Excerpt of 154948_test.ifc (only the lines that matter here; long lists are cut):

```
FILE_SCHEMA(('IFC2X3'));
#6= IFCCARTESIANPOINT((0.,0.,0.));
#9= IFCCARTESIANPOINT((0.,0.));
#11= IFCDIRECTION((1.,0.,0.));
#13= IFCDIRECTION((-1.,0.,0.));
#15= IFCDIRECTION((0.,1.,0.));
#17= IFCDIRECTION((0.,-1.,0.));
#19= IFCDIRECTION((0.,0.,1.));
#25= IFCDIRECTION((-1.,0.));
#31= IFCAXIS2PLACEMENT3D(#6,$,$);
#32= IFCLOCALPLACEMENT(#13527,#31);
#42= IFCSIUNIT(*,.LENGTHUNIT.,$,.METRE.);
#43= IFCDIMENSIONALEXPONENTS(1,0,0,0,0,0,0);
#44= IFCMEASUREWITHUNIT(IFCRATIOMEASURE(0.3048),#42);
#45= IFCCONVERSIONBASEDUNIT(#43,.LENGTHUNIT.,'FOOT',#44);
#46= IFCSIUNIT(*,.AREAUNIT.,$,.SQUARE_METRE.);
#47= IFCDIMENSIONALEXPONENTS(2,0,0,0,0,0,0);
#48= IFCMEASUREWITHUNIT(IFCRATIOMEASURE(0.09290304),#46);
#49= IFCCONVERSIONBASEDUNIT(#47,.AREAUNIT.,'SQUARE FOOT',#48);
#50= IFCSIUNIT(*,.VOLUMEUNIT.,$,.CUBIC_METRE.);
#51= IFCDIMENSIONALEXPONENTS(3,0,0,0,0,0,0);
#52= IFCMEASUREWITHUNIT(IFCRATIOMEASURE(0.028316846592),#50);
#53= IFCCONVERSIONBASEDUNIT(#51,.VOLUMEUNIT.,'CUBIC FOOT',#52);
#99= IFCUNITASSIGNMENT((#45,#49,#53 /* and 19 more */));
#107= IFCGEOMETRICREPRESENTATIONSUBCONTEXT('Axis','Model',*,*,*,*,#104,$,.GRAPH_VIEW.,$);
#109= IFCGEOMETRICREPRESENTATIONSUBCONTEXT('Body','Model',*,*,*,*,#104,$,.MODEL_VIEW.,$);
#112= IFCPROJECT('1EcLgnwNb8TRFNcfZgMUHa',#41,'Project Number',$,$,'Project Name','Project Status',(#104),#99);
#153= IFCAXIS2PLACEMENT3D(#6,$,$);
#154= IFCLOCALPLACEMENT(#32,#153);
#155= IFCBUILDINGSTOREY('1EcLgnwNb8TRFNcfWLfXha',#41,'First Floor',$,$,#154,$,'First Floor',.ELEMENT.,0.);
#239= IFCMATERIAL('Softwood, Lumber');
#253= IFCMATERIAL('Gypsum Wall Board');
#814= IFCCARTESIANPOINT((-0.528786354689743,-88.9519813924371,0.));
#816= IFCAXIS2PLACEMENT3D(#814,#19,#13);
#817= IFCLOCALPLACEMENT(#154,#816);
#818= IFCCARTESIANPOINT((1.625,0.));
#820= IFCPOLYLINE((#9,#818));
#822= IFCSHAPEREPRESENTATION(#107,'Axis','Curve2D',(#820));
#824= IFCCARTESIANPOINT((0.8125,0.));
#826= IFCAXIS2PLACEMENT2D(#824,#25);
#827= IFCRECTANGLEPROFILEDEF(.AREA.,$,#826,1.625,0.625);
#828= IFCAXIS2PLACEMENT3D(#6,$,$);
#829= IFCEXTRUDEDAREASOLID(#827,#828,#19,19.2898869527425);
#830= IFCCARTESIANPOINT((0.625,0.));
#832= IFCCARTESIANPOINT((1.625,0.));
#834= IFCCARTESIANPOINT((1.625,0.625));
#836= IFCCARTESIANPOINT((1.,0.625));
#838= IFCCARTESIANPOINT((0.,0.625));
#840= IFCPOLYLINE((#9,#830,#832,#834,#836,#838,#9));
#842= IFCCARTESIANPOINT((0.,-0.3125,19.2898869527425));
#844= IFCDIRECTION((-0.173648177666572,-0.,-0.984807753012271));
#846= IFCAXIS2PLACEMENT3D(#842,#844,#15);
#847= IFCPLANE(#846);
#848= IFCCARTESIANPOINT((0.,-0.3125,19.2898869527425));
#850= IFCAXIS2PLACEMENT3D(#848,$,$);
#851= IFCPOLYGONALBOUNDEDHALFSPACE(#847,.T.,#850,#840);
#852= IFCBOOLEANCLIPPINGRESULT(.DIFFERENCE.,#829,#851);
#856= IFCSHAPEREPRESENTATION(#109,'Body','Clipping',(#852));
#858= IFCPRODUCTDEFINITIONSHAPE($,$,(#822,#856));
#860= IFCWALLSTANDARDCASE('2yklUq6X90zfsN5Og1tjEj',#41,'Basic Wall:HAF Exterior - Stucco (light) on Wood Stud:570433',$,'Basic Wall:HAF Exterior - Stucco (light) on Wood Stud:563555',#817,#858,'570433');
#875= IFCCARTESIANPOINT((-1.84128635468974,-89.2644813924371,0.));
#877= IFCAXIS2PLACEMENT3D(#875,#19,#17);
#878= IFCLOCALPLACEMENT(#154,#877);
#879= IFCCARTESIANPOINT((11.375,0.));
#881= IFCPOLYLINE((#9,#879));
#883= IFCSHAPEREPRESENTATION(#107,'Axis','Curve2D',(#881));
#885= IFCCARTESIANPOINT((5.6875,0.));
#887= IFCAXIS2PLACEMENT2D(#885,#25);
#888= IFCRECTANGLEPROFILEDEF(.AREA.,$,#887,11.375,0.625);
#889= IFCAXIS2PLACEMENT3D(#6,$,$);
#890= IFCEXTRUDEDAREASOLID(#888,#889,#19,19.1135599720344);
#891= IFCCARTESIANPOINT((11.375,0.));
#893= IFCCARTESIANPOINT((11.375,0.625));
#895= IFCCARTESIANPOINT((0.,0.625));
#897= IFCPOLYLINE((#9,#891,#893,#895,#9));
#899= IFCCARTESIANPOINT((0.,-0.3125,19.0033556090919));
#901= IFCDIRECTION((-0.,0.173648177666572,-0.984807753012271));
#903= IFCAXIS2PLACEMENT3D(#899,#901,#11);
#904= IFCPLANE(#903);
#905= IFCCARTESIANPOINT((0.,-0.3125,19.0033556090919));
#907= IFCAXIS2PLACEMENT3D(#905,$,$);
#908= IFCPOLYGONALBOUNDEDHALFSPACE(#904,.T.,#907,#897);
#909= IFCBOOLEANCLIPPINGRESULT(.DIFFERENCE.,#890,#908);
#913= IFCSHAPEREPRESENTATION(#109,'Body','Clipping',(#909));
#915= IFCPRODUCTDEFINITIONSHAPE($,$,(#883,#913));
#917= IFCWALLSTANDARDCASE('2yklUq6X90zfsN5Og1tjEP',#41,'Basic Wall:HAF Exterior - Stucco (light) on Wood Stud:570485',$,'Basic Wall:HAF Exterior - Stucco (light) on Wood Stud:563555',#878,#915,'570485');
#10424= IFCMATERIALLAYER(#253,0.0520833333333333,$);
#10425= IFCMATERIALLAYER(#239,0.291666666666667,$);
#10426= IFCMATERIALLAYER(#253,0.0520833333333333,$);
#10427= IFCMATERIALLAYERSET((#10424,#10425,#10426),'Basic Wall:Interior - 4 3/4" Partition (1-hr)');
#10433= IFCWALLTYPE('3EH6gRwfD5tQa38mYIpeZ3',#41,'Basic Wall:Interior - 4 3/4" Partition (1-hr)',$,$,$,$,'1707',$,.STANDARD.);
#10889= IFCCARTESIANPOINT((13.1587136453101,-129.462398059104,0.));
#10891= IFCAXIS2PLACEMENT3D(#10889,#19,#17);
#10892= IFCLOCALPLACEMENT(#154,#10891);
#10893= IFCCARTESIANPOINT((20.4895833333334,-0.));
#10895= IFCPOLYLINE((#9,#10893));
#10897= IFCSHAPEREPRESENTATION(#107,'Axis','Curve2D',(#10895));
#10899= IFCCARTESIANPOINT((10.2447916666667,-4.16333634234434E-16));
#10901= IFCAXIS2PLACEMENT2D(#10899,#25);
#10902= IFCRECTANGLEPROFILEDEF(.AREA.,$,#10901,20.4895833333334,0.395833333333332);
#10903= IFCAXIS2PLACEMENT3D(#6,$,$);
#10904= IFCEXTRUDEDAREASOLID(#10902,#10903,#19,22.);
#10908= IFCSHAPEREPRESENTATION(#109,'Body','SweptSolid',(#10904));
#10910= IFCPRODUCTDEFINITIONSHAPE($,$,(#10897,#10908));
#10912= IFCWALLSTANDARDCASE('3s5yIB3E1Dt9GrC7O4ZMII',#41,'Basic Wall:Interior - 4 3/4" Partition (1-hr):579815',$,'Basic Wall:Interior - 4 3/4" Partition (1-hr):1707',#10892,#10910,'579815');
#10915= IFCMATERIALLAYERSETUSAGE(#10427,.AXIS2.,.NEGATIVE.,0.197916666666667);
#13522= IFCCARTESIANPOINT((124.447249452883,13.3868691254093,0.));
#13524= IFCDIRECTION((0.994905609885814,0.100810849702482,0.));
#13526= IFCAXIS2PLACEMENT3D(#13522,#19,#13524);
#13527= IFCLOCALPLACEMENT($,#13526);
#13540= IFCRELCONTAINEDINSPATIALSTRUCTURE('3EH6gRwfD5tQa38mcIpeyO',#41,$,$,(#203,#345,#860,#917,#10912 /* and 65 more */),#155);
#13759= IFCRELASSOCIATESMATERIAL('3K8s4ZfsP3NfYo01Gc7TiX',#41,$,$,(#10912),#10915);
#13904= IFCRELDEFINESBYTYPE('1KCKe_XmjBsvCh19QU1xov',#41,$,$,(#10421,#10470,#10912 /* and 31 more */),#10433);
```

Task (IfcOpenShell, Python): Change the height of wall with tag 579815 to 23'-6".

```python
import ifcopenshell
import ifcopenshell.geom
import ifcopenshell.util.representation
import ifcopenshell.util.shape
import ifcopenshell.util.unit

model = ifcopenshell.open("154948_test.ifc")
unit_scale = ifcopenshell.util.unit.calculate_unit_scale(model)
settings = ifcopenshell.geom.settings()


def volume(element):
    """Net volume in cubic metres, openings subtracted."""
    shape = ifcopenshell.geom.create_shape(settings, element)
    return ifcopenshell.util.shape.get_volume(shape.geometry)


wall = model.by_id(10912)
before = volume(wall)

body = ifcopenshell.util.representation.get_representation(wall, "Model", "Body")
solid = body.Items[0]
old_height = solid.Depth
solid.Depth = 282 * 0.0254 / unit_scale
after = volume(wall)

print(f"height {old_height:g} -> {solid.Depth:g}, volume {before:.3f} -> {after:.3f} m3")

model.write("154948_test-out.ifc")
```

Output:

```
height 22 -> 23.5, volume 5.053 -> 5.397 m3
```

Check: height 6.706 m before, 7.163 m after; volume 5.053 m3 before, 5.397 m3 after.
